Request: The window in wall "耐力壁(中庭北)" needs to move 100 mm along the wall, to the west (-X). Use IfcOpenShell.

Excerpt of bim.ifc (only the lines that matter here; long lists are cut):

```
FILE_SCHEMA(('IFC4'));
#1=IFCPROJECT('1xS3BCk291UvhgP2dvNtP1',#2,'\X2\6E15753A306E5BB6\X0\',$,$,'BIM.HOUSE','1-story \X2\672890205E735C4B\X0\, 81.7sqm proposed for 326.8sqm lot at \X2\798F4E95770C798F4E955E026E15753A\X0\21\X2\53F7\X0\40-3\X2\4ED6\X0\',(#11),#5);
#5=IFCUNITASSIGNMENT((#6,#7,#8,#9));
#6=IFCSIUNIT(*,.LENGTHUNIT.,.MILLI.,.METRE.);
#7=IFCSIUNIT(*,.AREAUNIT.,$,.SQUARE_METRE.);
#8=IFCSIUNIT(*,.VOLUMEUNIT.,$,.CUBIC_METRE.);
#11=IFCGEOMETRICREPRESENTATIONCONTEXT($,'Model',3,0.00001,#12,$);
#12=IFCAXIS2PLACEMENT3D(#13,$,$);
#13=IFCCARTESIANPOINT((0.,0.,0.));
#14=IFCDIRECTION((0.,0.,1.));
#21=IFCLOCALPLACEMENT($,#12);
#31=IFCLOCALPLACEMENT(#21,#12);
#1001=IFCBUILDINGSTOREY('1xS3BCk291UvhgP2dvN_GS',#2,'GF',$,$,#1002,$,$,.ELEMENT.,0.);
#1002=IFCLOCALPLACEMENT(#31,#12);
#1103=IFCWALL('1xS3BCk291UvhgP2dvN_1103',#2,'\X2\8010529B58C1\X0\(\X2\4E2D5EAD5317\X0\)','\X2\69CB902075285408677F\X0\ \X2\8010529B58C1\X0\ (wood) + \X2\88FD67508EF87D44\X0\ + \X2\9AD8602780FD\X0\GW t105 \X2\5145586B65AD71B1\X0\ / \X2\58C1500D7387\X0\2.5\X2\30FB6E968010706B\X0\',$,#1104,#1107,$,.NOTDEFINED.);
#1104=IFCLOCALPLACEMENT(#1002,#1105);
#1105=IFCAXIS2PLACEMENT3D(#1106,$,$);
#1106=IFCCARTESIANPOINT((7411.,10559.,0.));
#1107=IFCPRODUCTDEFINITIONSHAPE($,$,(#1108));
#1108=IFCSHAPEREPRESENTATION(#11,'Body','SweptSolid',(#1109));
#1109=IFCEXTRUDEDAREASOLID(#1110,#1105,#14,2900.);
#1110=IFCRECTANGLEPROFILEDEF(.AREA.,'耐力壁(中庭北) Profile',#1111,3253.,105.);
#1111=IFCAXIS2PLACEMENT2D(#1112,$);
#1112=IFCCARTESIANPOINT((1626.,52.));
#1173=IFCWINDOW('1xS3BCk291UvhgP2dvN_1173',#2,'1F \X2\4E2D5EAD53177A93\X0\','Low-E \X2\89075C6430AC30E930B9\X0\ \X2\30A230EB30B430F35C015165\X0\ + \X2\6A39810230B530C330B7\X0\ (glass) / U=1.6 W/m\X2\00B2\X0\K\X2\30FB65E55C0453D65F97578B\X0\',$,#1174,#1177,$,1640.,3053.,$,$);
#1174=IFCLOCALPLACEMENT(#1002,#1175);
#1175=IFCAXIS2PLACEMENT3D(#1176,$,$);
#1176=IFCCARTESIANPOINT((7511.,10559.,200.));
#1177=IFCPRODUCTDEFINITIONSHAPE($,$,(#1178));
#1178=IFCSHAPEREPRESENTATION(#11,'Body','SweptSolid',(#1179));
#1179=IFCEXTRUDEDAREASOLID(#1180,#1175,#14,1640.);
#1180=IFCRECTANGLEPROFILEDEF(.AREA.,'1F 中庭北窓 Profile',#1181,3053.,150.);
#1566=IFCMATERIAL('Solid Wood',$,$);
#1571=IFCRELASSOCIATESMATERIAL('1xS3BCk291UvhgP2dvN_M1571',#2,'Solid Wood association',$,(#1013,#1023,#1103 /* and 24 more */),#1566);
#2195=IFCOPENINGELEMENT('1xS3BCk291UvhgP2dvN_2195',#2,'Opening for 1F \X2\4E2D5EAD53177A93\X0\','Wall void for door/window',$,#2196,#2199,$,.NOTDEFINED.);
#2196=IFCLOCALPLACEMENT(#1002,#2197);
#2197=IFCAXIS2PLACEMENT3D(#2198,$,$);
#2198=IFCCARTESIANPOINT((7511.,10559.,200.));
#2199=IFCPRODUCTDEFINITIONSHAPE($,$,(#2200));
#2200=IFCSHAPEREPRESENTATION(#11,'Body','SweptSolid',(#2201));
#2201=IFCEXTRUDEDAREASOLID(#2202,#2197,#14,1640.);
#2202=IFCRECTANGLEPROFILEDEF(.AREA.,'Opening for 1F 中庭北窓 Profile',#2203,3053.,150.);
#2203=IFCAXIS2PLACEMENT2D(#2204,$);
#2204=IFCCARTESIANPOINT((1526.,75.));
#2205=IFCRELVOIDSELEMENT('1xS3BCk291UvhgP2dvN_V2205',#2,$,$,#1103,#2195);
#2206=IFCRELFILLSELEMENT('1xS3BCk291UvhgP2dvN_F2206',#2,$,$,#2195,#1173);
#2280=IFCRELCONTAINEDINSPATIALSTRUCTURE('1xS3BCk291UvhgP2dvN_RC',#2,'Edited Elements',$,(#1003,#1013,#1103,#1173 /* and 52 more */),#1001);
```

```python
import ifcopenshell
import ifcopenshell.api.geometry
import ifcopenshell.util.placement
import ifcopenshell.util.unit

model = ifcopenshell.open("bim.ifc")
unit_scale = ifcopenshell.util.unit.calculate_unit_scale(model)

window = model.by_guid("1xS3BCk291UvhgP2dvN_1173")
opening = window.FillsVoids[0].RelatingOpeningElement
wall = opening.VoidsElements[0].RelatingBuildingElement

wall_matrix = ifcopenshell.util.placement.get_local_placement(wall.ObjectPlacement)
shift = wall_matrix[:3, 0] * -0.1 / unit_scale
before = ifcopenshell.util.placement.get_local_placement(window.ObjectPlacement)[:3, 3].copy()

# The window is not placed relative to its opening, so move both.
for product in (opening, window):
    matrix = ifcopenshell.util.placement.get_local_placement(product.ObjectPlacement)
    matrix[:3, 3] += shift
    ifcopenshell.api.geometry.edit_object_placement(model, product=product, matrix=matrix, is_si=False)

after = ifcopenshell.util.placement.get_local_placement(window.ObjectPlacement)[:3, 3]
print("window moved by", (after - before).round(3) + 0.0)

model.write("bim_updated.ifc")
```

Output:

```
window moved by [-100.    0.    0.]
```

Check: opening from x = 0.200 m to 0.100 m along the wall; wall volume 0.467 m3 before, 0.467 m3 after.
